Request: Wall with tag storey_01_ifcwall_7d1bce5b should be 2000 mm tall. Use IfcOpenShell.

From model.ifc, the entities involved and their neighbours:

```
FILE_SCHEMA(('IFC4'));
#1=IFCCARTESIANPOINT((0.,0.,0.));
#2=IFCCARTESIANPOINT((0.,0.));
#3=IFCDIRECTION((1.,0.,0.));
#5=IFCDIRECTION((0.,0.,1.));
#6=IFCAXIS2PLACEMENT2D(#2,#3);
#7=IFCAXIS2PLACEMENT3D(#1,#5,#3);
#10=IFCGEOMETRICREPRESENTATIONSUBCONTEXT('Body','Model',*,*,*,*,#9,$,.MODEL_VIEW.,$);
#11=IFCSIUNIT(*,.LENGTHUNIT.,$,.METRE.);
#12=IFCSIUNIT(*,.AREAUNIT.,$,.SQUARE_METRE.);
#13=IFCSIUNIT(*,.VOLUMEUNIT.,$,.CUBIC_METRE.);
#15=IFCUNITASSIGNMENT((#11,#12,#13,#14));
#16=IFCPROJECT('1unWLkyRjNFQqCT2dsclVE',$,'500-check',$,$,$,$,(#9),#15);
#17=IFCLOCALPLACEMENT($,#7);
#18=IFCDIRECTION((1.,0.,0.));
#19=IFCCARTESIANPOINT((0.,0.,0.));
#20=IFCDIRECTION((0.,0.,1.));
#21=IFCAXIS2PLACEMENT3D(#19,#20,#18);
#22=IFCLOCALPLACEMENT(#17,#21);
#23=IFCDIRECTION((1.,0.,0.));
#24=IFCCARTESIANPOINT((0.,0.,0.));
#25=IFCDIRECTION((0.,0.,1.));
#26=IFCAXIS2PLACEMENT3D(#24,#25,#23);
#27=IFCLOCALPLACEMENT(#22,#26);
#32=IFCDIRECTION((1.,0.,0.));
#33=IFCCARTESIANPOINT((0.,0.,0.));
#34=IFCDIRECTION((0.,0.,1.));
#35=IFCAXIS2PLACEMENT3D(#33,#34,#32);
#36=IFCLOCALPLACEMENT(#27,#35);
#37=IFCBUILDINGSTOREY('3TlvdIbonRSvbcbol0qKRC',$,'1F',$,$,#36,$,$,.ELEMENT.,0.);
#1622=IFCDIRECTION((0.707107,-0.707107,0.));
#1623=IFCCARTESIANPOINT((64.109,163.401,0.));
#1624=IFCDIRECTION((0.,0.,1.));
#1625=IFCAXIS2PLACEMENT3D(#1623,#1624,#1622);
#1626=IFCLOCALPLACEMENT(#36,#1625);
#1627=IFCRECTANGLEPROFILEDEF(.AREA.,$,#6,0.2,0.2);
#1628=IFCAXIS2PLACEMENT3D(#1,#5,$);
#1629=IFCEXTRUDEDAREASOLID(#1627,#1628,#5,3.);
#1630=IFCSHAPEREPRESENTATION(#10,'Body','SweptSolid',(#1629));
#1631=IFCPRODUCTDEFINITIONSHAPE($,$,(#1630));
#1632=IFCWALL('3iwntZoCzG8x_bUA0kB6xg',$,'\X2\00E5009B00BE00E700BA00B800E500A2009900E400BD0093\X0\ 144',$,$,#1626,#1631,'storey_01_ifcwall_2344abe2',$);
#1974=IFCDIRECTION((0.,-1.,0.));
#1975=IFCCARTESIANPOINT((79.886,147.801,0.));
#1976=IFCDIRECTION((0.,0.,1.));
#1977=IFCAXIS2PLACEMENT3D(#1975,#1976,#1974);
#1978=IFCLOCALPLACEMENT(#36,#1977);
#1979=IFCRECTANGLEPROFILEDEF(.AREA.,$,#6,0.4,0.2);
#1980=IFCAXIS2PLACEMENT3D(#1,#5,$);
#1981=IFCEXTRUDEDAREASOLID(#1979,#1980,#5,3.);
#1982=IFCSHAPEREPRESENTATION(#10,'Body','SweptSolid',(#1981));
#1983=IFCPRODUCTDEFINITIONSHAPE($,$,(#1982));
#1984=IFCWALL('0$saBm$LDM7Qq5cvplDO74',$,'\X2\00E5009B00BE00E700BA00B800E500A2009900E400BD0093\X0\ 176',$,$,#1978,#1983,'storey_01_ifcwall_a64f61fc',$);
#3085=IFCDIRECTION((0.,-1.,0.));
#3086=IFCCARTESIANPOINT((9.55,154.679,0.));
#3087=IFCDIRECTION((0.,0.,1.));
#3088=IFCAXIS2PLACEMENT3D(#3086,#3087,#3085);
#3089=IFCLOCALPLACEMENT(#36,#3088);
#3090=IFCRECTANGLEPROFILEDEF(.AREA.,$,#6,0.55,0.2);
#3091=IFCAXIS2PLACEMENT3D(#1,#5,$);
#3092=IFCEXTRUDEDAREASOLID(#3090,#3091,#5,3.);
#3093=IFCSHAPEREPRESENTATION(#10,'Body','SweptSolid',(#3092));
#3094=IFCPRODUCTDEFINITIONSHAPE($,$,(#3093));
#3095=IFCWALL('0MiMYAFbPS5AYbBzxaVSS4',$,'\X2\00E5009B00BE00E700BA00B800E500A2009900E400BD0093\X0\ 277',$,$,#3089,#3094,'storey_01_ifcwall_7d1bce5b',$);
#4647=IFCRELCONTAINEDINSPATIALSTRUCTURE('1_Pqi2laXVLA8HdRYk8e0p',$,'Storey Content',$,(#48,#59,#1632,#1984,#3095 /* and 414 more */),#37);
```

```python
import ifcopenshell
import ifcopenshell.geom
import ifcopenshell.util.representation
import ifcopenshell.util.shape

model = ifcopenshell.open("model.ifc")
settings = ifcopenshell.geom.settings()


def volume(element):
    """Net volume in cubic metres, openings subtracted."""
    shape = ifcopenshell.geom.create_shape(settings, element)
    return ifcopenshell.util.shape.get_volume(shape.geometry)


wall = model.by_guid("0MiMYAFbPS5AYbBzxaVSS4")
before = volume(wall)

body = ifcopenshell.util.representation.get_representation(wall, "Model", "Body")
solid = body.Items[0]
old_height = solid.Depth
solid.Depth = 2.0
after = volume(wall)

print(f"height {old_height:g} -> {solid.Depth:g}, volume {before:.3f} -> {after:.3f} m3")

model.write("model_edited.ifc")
```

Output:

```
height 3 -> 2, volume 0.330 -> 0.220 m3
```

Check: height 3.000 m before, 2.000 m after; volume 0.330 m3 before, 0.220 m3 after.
